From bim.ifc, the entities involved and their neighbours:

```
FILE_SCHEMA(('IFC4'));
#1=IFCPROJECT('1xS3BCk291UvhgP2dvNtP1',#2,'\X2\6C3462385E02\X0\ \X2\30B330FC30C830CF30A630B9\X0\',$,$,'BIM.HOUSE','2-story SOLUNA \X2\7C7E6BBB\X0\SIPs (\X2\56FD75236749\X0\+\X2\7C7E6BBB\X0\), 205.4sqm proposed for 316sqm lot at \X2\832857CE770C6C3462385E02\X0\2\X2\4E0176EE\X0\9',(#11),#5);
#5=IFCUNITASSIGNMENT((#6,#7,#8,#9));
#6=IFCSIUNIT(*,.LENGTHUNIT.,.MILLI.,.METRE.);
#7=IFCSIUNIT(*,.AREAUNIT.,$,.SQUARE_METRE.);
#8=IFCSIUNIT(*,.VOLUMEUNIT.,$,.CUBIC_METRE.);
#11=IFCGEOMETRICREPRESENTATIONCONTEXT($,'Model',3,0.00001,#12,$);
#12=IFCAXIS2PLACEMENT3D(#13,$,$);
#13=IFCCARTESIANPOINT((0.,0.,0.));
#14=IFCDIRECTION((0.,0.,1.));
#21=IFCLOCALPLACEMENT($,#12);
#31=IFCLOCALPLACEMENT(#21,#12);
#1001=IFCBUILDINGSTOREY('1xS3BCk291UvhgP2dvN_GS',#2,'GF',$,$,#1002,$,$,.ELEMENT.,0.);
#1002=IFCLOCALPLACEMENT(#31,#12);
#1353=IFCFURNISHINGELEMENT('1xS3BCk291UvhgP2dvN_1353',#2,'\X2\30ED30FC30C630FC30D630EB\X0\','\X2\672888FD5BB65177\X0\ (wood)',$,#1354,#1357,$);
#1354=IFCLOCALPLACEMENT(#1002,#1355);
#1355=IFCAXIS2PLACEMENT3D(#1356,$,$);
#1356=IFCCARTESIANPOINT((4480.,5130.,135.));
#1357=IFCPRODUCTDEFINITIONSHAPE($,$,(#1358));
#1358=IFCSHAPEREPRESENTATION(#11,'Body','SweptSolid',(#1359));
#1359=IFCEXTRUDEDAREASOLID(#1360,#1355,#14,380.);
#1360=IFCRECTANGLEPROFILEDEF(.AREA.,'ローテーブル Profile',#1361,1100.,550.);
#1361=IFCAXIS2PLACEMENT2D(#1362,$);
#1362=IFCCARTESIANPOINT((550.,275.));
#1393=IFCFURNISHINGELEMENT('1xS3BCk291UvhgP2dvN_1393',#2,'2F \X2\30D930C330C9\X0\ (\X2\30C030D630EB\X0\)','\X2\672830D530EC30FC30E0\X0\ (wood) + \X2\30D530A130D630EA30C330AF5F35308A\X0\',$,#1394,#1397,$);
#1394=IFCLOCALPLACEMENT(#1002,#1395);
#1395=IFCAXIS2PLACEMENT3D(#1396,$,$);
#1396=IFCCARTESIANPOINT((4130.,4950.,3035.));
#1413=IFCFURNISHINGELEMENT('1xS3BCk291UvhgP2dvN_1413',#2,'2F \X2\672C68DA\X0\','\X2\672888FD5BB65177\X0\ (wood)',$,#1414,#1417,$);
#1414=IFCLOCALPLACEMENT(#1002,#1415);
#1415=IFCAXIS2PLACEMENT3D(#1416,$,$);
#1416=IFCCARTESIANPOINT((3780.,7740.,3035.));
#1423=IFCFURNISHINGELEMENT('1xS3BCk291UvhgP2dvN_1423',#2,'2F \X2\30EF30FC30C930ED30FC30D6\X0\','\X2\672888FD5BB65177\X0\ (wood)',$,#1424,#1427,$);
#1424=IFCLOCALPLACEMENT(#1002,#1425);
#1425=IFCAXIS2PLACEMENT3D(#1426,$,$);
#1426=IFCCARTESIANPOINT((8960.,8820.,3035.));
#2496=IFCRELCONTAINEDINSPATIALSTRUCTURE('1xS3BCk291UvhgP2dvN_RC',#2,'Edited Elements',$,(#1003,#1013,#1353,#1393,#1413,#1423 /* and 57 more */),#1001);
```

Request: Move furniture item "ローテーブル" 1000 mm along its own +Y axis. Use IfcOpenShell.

```python
import ifcopenshell
import ifcopenshell.api.geometry
import ifcopenshell.util.placement
import ifcopenshell.util.unit

model = ifcopenshell.open("bim.ifc")
unit_scale = ifcopenshell.util.unit.calculate_unit_scale(model)

item = model.by_guid("1xS3BCk291UvhgP2dvN_1353")
matrix = ifcopenshell.util.placement.get_local_placement(item.ObjectPlacement)
matrix[:3, 3] += matrix[:3, 1] * 1 / unit_scale
ifcopenshell.api.geometry.edit_object_placement(model, product=item, matrix=matrix, is_si=False)

print(ifcopenshell.util.placement.get_local_placement(item.ObjectPlacement).round(3) + 0.0)

model.write("bim_rev.ifc")
```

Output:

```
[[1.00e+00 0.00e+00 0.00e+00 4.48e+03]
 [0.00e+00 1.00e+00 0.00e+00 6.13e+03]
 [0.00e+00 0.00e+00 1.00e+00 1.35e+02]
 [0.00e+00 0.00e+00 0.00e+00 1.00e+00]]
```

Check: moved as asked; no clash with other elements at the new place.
